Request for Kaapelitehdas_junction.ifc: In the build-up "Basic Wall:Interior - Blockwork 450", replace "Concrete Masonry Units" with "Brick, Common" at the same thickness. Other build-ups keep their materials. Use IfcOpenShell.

First a look at what the model holds.

```python
import ifcopenshell
import ifcopenshell.util.element

model = ifcopenshell.open("Kaapelitehdas_junction.ifc")
print(model.schema)
for layer_set in model.by_type("IfcMaterialLayerSet"):
    if layer_set.LayerSetName == "Basic Wall:Interior - Blockwork 450":
        for layer in layer_set.MaterialLayers:
            print(layer.id(), layer.Material and layer.Material.Name, layer.LayerThickness, sep=" | ")
        print(len(ifcopenshell.util.element.get_elements_by_material(model, layer_set)), "elements and types use it")
print(sorted(m.Name for m in model.by_type("IfcMaterial") if m.Name)[:60])
```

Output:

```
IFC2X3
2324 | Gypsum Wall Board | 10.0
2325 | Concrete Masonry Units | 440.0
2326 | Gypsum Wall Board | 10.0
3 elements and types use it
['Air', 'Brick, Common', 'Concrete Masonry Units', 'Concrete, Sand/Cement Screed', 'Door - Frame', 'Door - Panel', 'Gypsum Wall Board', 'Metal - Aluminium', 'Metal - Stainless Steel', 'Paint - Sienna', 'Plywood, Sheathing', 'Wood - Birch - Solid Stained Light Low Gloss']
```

```python
import ifcopenshell
import ifcopenshell.api.material

model = ifcopenshell.open("Kaapelitehdas_junction.ifc")

layer_set = next(s for s in model.by_type("IfcMaterialLayerSet") if s.LayerSetName == "Basic Wall:Interior - Blockwork 450")
layer = next(l for l in layer_set.MaterialLayers if l.Material and l.Material.Name == "Concrete Masonry Units")
material = next(m for m in model.by_type("IfcMaterial") if m.Name == "Brick, Common")

# Point this one layer at the other material; renaming the old one would change it everywhere.
ifcopenshell.api.material.edit_layer(model, layer=layer, attributes={}, material=material)

print([l.Material.Name if l.Material else None for l in layer_set.MaterialLayers])

model.write("Kaapelitehdas_junction_edited.ifc")
```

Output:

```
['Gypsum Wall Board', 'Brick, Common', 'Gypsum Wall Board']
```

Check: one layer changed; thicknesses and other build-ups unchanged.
